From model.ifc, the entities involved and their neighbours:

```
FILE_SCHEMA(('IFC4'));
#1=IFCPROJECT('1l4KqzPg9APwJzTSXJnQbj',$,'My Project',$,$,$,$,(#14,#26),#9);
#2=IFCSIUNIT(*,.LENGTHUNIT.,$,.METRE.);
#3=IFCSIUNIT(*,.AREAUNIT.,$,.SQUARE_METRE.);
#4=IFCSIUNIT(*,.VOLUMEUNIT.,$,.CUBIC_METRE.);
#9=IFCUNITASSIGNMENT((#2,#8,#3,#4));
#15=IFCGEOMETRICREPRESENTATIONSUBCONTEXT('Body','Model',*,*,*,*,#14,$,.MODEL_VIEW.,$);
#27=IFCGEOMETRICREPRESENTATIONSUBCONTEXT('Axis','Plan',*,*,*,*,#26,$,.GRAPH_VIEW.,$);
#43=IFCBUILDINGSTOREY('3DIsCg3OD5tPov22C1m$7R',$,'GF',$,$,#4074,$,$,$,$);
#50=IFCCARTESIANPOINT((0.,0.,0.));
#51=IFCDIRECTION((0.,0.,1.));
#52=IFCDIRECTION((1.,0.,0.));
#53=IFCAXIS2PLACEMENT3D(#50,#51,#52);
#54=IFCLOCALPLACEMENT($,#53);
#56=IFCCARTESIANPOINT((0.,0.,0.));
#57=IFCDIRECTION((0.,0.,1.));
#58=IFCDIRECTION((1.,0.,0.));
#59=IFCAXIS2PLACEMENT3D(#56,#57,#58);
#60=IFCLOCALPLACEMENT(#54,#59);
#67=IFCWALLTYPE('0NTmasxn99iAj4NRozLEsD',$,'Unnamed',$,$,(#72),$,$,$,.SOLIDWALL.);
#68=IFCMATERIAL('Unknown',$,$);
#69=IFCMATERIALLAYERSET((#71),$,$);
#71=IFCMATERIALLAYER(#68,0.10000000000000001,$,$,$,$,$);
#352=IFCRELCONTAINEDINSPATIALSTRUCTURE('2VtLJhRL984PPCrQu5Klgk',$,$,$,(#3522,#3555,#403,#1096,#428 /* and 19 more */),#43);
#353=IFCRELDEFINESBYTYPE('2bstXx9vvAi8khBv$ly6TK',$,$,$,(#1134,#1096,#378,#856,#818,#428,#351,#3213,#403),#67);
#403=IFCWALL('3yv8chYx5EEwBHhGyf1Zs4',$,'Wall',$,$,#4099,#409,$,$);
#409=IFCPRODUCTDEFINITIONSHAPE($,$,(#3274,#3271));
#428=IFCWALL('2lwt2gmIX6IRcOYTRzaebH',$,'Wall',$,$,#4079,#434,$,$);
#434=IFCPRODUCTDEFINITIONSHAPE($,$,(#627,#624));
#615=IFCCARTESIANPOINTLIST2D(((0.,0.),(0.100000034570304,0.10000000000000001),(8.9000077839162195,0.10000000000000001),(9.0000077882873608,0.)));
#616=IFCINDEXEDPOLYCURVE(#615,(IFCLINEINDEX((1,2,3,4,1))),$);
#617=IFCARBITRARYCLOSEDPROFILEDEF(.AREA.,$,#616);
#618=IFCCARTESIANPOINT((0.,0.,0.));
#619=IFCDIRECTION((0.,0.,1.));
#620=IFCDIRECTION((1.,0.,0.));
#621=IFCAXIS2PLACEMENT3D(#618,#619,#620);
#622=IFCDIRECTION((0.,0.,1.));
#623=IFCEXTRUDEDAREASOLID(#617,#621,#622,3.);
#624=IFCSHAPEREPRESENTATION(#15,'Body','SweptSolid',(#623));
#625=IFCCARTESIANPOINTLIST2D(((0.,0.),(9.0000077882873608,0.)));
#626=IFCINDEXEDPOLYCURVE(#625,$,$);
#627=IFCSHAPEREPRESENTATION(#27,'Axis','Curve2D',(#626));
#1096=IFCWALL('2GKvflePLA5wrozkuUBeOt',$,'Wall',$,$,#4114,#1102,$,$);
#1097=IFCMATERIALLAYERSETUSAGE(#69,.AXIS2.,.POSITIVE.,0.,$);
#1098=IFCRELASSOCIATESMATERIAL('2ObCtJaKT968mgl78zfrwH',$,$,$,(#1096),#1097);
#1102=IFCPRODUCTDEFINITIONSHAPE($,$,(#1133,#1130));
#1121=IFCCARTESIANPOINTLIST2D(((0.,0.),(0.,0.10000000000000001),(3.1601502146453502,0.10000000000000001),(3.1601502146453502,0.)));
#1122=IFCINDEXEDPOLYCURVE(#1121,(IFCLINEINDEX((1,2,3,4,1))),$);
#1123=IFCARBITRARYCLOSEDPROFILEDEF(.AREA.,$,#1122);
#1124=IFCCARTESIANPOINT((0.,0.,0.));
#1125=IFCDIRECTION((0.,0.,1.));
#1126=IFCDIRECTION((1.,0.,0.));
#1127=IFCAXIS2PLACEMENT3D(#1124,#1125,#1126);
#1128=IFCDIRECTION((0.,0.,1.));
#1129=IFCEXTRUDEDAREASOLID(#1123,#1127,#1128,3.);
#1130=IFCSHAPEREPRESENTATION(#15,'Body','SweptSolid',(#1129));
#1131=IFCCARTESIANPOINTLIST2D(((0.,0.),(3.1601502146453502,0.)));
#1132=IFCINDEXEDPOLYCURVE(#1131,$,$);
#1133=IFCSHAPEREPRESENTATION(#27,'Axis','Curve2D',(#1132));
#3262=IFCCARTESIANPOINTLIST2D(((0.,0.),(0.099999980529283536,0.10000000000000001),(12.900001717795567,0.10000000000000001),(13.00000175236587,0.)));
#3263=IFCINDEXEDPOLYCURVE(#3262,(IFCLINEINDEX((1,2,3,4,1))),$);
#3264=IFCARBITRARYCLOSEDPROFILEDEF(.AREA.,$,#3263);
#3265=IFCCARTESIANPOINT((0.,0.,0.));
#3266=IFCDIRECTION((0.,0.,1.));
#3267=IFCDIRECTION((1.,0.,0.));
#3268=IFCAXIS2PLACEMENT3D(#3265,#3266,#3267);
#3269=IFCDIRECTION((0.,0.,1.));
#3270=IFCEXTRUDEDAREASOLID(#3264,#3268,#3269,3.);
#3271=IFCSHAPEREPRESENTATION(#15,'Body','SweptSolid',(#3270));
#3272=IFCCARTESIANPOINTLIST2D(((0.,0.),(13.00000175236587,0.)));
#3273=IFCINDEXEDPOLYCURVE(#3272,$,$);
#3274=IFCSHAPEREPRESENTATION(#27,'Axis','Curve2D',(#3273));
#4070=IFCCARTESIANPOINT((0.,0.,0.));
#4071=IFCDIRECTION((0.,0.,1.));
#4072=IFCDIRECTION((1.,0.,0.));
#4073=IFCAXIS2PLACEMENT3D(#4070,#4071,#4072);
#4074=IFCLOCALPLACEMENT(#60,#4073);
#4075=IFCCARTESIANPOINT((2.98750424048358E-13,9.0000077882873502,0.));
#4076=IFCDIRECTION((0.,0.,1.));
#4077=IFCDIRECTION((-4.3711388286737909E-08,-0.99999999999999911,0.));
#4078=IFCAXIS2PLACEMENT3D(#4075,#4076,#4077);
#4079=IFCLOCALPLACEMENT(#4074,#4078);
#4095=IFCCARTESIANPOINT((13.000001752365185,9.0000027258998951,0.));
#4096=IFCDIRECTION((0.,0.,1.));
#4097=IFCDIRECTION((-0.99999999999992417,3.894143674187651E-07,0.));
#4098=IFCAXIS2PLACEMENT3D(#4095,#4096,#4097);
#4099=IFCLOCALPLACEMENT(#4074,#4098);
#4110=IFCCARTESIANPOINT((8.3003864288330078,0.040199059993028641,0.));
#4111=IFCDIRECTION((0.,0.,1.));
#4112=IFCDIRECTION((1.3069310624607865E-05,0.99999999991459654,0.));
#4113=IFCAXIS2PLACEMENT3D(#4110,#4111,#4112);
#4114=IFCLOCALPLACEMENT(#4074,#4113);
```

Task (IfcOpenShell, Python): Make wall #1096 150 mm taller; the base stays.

```python
import ifcopenshell
import ifcopenshell.geom
import ifcopenshell.util.representation
import ifcopenshell.util.shape
import ifcopenshell.util.unit

model = ifcopenshell.open("model.ifc")
unit_scale = ifcopenshell.util.unit.calculate_unit_scale(model)
settings = ifcopenshell.geom.settings()


def volume(element):
    """Net volume in cubic metres, openings subtracted."""
    shape = ifcopenshell.geom.create_shape(settings, element)
    return ifcopenshell.util.shape.get_volume(shape.geometry)


wall = model.by_guid("2GKvflePLA5wrozkuUBeOt")
before = volume(wall)

body = ifcopenshell.util.representation.get_representation(wall, "Model", "Body")
solid = body.Items[0]
old_height = solid.Depth
solid.Depth += 0.15 / unit_scale
after = volume(wall)

print(f"height {old_height:g} -> {solid.Depth:g}, volume {before:.3f} -> {after:.3f} m3")

model.write("model_v2.ifc")
```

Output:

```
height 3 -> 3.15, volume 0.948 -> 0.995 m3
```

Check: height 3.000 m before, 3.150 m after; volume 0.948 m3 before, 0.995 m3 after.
